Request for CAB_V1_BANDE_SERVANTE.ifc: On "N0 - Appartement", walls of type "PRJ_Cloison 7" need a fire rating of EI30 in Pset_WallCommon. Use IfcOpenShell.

First a look at what the model holds.

```python
import ifcopenshell
import ifcopenshell.util.element

model = ifcopenshell.open("CAB_V1_BANDE_SERVANTE.ifc")
print(model.schema)
storey = next(s for s in model.by_type("IfcBuildingStorey") if s.Name == "N0 - Appartement")
walls = [e for e in ifcopenshell.util.element.get_decomposition(storey) if e.is_a("IfcWall")]
seen = {}
for e in walls:
    element_type = ifcopenshell.util.element.get_type(e)
    key = (element_type.Name if element_type != e and element_type else None, ifcopenshell.util.element.get_pset(e, "Pset_WallCommon", "FireRating"))
    seen[key] = seen.get(key, 0) + 1
for (name, value), count in sorted(seen.items(), key=str):
    print(count, "x", name, "|", value)
```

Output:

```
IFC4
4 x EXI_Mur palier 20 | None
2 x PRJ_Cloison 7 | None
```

```python
import ifcopenshell
import ifcopenshell.api.pset
import ifcopenshell.util.element

model = ifcopenshell.open("CAB_V1_BANDE_SERVANTE.ifc")

storey = next(s for s in model.by_type("IfcBuildingStorey") if s.Name == "N0 - Appartement")
walls = [e for e in ifcopenshell.util.element.get_decomposition(storey) if e.is_a("IfcWall")]

count = 0
for e in walls:
    element_type = ifcopenshell.util.element.get_type(e)
    if element_type in (None, e) or element_type.Name != "PRJ_Cloison 7":
        continue
    # add_pset returns the element's existing set when there is one.
    pset = ifcopenshell.api.pset.add_pset(model, product=e, name="Pset_WallCommon")
    ifcopenshell.api.pset.edit_pset(model, pset=pset, properties={"FireRating": "EI30"})
    count += 1

print(count, "walls updated")

model.write("CAB_V1_BANDE_SERVANTE_v2.ifc")
```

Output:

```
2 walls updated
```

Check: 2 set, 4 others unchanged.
